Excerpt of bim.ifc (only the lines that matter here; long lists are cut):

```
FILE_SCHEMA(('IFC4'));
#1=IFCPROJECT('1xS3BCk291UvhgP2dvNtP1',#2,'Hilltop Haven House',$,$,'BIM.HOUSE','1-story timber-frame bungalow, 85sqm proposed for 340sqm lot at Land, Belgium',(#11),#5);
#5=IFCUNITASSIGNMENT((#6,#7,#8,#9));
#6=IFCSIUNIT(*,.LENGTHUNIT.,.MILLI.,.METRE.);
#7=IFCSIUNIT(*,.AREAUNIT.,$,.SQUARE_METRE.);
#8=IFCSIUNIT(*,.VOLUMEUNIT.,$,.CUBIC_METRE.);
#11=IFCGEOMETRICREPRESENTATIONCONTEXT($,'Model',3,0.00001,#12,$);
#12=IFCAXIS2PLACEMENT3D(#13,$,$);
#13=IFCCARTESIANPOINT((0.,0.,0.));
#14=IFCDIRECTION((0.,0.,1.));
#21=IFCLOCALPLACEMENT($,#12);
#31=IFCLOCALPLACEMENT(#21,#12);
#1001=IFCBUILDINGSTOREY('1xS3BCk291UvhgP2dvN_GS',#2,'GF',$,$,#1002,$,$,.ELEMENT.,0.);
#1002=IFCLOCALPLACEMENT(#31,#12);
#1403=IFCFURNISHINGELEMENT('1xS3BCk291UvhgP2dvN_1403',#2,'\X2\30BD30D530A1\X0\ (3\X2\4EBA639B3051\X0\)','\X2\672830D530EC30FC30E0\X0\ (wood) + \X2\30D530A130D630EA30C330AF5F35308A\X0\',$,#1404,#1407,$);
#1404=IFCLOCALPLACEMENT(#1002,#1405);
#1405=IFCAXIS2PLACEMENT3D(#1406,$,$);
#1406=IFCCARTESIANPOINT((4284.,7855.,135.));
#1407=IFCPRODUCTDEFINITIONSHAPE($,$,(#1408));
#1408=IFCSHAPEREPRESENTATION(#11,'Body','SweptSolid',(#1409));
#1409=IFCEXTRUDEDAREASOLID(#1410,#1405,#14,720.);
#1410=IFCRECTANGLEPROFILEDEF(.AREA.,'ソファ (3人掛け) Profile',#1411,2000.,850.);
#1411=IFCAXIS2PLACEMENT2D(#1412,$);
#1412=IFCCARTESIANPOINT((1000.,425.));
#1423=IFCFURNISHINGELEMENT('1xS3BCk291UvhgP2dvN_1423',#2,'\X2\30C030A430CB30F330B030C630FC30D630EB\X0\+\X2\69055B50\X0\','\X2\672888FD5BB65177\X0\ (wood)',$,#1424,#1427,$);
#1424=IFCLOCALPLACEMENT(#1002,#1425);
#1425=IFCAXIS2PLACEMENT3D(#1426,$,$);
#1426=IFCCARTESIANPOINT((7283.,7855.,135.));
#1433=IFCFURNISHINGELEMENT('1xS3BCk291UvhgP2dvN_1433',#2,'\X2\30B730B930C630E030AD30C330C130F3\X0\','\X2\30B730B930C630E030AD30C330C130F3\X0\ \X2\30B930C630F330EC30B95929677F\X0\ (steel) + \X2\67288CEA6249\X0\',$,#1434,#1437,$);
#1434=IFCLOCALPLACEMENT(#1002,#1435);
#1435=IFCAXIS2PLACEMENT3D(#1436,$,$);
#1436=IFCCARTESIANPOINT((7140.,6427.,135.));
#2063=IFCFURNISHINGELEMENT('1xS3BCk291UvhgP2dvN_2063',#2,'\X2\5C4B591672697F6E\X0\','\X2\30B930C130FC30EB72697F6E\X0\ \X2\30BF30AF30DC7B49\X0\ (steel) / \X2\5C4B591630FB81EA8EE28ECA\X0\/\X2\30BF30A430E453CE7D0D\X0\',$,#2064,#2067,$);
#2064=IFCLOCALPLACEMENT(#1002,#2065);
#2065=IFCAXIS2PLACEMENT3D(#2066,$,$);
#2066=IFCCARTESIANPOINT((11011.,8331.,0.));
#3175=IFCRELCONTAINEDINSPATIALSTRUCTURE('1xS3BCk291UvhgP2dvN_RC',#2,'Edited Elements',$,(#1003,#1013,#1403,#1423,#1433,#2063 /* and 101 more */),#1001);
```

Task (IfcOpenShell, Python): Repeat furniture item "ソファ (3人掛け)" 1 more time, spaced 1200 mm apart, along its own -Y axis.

```python
import ifcopenshell
import ifcopenshell.api.geometry
import ifcopenshell.api.root
import ifcopenshell.util.element
import ifcopenshell.util.placement

model = ifcopenshell.open("bim.ifc")


def reuse_history(source, copy):
    """copy_class also copies each property set's owner history, people and application; keep the originals."""
    for rel in copy.IsDefinedBy:
        if rel.is_a("IfcRelDefinesByProperties") and (history := rel.RelatingPropertyDefinition.OwnerHistory):
            rel.RelatingPropertyDefinition.OwnerHistory = source.OwnerHistory
            ifcopenshell.util.element.remove_deep2(model, history)


source = model.by_guid("1xS3BCk291UvhgP2dvN_1403")
base = ifcopenshell.util.placement.get_local_placement(source.ObjectPlacement)
step = -base[:3, 1] * 1200.0

for i in range(1, 2):
    copy = ifcopenshell.api.root.copy_class(model, product=source)
    copy.Representation = ifcopenshell.util.element.copy_deep(
        model, source.Representation, exclude=["IfcGeometricRepresentationContext", "IfcRepresentationMap"]
    )
    reuse_history(source, copy)
    matrix = base.copy()
    matrix[:3, 3] += i * step
    print("added at", matrix[:3, 3].round(3) + 0.0)
    ifcopenshell.api.geometry.edit_object_placement(model, product=copy, matrix=matrix, is_si=False)

model.write("bim_v2.ifc")
```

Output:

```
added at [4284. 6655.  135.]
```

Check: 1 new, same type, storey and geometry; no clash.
